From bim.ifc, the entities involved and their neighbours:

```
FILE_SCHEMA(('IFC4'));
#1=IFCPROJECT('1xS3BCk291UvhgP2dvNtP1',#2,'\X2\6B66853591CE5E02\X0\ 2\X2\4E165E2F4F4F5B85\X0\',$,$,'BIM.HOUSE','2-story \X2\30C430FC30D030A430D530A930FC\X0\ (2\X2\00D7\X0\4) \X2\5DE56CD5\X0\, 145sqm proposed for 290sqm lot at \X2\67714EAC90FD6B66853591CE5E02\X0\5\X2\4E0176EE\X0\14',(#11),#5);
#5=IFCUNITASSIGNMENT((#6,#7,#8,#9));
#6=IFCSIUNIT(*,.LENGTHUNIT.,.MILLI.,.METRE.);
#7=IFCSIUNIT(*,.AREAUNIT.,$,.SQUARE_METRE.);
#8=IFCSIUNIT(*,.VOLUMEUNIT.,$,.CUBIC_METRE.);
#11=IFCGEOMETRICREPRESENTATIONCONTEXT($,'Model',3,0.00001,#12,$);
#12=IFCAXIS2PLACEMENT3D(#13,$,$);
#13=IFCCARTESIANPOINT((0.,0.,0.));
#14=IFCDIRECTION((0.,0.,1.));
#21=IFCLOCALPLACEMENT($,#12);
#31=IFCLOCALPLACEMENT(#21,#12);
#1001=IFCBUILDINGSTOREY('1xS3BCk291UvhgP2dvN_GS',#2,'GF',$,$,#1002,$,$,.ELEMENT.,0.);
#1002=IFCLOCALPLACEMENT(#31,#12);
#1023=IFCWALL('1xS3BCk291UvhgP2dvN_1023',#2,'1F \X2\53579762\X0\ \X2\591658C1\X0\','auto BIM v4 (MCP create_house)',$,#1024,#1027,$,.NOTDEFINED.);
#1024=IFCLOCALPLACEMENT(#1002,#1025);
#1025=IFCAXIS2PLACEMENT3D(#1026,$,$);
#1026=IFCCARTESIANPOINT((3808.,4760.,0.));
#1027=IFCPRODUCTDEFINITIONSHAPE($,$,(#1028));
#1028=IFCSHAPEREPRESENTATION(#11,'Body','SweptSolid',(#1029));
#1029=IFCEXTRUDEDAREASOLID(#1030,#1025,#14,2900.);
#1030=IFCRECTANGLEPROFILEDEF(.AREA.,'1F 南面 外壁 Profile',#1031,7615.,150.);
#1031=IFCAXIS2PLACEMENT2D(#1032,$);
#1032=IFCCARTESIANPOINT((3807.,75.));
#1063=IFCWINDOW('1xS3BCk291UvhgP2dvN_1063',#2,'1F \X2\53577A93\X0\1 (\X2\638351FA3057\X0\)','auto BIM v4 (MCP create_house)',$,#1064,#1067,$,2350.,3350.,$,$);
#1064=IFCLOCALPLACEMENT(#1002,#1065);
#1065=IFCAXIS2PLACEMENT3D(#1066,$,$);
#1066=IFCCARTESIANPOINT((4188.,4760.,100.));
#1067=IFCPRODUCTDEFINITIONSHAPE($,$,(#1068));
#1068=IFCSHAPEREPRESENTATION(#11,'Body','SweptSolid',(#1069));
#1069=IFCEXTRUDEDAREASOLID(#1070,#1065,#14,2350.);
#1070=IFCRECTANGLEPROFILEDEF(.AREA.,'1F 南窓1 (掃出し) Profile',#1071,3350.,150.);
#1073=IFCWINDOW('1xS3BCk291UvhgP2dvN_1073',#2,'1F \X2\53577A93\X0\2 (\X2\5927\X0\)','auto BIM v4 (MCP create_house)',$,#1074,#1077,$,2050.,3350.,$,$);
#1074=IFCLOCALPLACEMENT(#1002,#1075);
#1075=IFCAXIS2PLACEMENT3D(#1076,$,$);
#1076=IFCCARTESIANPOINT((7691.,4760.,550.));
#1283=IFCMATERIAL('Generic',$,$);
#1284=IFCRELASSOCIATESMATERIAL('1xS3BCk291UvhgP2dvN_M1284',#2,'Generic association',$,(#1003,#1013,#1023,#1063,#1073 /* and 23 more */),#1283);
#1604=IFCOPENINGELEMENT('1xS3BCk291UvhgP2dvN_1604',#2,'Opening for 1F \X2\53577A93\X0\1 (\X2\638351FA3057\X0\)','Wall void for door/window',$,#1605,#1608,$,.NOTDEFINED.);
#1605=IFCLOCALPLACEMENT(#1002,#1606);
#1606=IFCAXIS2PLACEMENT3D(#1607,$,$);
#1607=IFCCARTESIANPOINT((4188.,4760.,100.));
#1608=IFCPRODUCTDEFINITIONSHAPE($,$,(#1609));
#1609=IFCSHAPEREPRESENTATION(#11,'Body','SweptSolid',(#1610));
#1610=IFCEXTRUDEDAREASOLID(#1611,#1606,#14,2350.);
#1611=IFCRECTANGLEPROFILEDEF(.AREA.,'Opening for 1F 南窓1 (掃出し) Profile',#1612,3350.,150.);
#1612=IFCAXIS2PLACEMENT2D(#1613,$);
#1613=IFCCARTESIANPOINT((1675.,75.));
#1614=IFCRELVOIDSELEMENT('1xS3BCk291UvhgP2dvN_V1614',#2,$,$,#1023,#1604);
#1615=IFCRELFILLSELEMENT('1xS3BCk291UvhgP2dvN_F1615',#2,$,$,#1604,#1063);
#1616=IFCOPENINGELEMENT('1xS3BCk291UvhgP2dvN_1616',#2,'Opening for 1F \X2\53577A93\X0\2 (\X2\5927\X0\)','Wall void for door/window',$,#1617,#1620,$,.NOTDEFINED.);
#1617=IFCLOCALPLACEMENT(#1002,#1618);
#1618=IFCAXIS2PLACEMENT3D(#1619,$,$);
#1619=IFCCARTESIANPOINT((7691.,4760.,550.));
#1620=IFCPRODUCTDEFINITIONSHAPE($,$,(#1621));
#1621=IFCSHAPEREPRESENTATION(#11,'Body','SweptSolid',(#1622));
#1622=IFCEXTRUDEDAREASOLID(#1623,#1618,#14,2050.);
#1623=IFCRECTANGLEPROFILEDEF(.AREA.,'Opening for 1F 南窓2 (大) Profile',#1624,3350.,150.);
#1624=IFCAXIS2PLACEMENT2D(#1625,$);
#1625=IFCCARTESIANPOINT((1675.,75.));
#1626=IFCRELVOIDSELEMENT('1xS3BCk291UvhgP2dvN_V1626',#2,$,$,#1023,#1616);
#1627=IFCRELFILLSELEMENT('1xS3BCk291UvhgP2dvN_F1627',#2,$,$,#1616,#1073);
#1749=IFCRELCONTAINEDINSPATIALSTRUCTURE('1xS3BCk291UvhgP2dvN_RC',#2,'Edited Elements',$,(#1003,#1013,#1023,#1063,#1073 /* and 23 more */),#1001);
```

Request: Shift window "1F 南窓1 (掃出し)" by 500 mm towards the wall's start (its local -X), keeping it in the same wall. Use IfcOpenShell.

```python
import ifcopenshell
import ifcopenshell.api.geometry
import ifcopenshell.util.placement

model = ifcopenshell.open("bim.ifc")

window = model.by_id(1063)
opening = window.FillsVoids[0].RelatingOpeningElement
wall = opening.VoidsElements[0].RelatingBuildingElement

wall_matrix = ifcopenshell.util.placement.get_local_placement(wall.ObjectPlacement)
shift = wall_matrix[:3, 0] * -500.0
before = ifcopenshell.util.placement.get_local_placement(window.ObjectPlacement)[:3, 3].copy()

# The window is not placed relative to its opening, so move both.
for product in (opening, window):
    matrix = ifcopenshell.util.placement.get_local_placement(product.ObjectPlacement)
    matrix[:3, 3] += shift
    ifcopenshell.api.geometry.edit_object_placement(model, product=product, matrix=matrix, is_si=False)

after = ifcopenshell.util.placement.get_local_placement(window.ObjectPlacement)[:3, 3]
print("window moved by", (after - before).round(3) + 0.0)

model.write("bim_updated.ifc")
```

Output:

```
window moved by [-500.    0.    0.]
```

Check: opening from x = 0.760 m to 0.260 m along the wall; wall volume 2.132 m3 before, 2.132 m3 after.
